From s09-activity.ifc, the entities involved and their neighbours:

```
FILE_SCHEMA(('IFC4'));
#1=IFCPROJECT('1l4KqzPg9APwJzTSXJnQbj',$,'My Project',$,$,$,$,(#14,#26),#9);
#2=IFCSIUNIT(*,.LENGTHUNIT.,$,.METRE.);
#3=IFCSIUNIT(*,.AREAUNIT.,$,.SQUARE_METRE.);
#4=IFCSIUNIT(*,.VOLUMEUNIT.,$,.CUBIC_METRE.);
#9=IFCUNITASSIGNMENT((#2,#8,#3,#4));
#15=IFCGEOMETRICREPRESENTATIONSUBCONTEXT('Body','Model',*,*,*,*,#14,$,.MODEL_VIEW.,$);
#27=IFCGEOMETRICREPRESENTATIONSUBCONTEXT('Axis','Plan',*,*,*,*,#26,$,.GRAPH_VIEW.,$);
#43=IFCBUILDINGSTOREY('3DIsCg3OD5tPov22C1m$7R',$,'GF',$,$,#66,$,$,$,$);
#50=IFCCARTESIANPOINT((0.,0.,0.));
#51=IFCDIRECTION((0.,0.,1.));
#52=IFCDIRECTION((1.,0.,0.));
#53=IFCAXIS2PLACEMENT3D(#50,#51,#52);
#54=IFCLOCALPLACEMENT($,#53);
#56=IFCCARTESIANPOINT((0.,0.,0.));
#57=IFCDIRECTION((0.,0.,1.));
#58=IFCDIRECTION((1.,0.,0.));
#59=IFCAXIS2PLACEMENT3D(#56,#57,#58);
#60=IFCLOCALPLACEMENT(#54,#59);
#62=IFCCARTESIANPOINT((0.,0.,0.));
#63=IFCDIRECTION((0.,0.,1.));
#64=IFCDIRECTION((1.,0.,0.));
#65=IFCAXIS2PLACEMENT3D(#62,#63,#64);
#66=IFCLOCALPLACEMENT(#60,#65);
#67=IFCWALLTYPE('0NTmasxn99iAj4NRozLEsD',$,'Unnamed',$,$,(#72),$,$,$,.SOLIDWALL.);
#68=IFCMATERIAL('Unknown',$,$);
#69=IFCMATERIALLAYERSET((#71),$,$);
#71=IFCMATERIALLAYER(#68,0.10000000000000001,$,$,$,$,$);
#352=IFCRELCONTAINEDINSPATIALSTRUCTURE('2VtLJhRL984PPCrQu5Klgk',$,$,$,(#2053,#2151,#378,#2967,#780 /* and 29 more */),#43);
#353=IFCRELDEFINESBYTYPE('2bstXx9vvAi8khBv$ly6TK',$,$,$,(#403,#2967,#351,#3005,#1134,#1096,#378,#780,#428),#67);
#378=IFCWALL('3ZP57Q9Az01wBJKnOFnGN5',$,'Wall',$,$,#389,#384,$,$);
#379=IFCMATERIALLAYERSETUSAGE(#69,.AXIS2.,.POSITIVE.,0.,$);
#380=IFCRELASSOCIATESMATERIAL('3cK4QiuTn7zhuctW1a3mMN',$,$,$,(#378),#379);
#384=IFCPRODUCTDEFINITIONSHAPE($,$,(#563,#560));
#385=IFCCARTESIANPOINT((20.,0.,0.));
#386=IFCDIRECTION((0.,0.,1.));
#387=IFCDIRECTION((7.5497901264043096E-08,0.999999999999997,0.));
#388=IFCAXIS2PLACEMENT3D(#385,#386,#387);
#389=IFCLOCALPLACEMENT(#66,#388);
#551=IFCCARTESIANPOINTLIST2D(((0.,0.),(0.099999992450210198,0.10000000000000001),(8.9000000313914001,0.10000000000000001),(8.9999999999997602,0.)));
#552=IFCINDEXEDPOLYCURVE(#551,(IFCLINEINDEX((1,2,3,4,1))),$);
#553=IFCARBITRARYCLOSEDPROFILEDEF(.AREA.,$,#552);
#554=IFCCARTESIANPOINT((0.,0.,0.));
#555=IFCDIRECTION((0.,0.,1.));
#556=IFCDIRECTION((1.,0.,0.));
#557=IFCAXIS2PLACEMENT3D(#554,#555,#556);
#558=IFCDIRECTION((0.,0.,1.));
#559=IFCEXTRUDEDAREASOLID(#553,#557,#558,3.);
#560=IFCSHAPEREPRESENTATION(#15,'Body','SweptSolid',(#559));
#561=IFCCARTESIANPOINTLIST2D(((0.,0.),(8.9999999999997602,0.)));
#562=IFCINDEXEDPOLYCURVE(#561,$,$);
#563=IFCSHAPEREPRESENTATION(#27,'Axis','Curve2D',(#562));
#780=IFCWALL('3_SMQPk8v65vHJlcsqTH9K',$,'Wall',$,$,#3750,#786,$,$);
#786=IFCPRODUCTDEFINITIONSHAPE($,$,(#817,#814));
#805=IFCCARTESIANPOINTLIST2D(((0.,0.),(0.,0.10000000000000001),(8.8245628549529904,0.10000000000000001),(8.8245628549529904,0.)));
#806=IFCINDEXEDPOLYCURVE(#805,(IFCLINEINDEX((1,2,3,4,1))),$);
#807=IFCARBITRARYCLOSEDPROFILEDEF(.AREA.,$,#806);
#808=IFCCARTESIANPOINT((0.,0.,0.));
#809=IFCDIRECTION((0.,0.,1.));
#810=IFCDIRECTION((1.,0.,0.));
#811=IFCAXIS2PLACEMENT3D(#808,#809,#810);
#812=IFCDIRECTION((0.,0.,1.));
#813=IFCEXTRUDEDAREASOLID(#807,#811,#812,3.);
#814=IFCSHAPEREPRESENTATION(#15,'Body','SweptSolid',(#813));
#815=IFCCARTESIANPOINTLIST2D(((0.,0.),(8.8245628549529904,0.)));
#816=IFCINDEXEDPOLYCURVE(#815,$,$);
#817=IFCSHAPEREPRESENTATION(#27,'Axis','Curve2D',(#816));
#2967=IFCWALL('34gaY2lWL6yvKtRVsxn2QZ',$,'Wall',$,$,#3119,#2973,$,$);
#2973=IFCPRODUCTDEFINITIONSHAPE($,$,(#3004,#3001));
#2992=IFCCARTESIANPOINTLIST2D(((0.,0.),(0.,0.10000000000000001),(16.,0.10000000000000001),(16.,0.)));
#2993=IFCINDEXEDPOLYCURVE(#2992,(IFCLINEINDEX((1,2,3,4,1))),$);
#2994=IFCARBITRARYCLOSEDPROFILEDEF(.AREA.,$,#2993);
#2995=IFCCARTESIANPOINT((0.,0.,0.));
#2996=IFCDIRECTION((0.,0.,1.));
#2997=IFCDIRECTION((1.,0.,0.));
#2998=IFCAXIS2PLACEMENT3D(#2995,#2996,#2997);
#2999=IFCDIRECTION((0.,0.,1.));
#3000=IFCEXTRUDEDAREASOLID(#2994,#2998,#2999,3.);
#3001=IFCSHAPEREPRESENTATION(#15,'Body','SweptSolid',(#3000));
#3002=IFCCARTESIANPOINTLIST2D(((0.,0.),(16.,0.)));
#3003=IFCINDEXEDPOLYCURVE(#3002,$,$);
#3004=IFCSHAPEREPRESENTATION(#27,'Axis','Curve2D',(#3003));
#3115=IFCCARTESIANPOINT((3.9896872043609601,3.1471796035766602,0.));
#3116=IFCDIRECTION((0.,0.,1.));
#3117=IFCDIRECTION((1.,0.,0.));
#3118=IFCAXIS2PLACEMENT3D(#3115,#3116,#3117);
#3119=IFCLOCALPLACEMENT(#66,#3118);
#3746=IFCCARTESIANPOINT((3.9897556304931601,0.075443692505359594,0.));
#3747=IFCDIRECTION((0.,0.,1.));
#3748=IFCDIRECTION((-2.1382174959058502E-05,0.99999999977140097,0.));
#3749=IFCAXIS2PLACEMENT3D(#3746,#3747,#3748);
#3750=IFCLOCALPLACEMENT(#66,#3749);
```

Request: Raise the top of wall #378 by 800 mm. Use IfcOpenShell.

```python
import ifcopenshell
import ifcopenshell.geom
import ifcopenshell.util.representation
import ifcopenshell.util.shape
import ifcopenshell.util.unit

model = ifcopenshell.open("s09-activity.ifc")
unit_scale = ifcopenshell.util.unit.calculate_unit_scale(model)
settings = ifcopenshell.geom.settings()


def volume(element):
    """Net volume in cubic metres, openings subtracted."""
    shape = ifcopenshell.geom.create_shape(settings, element)
    return ifcopenshell.util.shape.get_volume(shape.geometry)


wall = model.by_guid("3ZP57Q9Az01wBJKnOFnGN5")
before = volume(wall)

body = ifcopenshell.util.representation.get_representation(wall, "Model", "Body")
solid = body.Items[0]
old_height = solid.Depth
solid.Depth += 0.8 / unit_scale
after = volume(wall)

print(f"height {old_height:g} -> {solid.Depth:g}, volume {before:.3f} -> {after:.3f} m3")

model.write("s09-activity_edited.ifc")
```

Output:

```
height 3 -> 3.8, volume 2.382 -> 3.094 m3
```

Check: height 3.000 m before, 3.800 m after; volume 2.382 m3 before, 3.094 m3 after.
